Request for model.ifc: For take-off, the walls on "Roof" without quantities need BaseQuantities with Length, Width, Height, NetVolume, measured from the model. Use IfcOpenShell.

First a look at what the model holds.

```python
import ifcopenshell
import ifcopenshell.util.element
import ifcopenshell.util.unit

model = ifcopenshell.open("model.ifc")
print(model.schema)
for unit_type in ("LENGTHUNIT", "AREAUNIT", "VOLUMEUNIT"):
    print(unit_type, ifcopenshell.util.unit.calculate_unit_scale(model, unit_type))
storey = next(s for s in model.by_type("IfcBuildingStorey") if s.Name == "Roof")
walls = [e for e in ifcopenshell.util.element.get_decomposition(storey) if e.is_a("IfcWall")]
for e in sorted(walls, key=lambda e: e.id()):
    print(e.id(), e.is_a(), e.Name, list(ifcopenshell.util.element.get_psets(e, qtos_only=True)), sep=" | ")
```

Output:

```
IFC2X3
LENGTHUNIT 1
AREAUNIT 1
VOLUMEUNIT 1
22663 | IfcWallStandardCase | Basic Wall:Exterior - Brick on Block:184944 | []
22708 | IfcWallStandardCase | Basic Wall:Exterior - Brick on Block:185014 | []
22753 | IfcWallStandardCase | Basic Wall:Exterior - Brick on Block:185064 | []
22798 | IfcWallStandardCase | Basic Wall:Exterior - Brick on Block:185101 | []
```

```python
import ifcopenshell
import ifcopenshell.api.pset
import ifcopenshell.geom
import ifcopenshell.util.element
import ifcopenshell.util.shape
import ifcopenshell.util.unit

model = ifcopenshell.open("model.ifc")
unit_scale = ifcopenshell.util.unit.calculate_unit_scale(model)
volume_scale = ifcopenshell.util.unit.calculate_unit_scale(model, "VOLUMEUNIT")
settings = ifcopenshell.geom.settings()

storey = next(s for s in model.by_type("IfcBuildingStorey") if s.Name == "Roof")
walls = [e for e in ifcopenshell.util.element.get_decomposition(storey) if e.is_a("IfcWall")]

for e in sorted(walls, key=lambda e: e.id()):
    if ifcopenshell.util.element.get_psets(e, qtos_only=True, should_inherit=False):
        continue
    # Geometry comes back in metres, in the element's own axes.
    shape = ifcopenshell.geom.create_shape(settings, e)
    values = {
        "Length": ifcopenshell.util.shape.get_x(shape.geometry) / unit_scale,
        "Width": ifcopenshell.util.shape.get_y(shape.geometry) / unit_scale,
        "Height": ifcopenshell.util.shape.get_z(shape.geometry) / unit_scale,
        "NetVolume": ifcopenshell.util.shape.get_volume(shape.geometry) / volume_scale,
    }
    qto = ifcopenshell.api.pset.add_qto(model, product=e, name="BaseQuantities")
    ifcopenshell.api.pset.edit_qto(model, qto=qto, properties=values)
    print(e.id(), {k: round(v, 3) for k, v in values.items()})

model.write("model-out.ifc")
```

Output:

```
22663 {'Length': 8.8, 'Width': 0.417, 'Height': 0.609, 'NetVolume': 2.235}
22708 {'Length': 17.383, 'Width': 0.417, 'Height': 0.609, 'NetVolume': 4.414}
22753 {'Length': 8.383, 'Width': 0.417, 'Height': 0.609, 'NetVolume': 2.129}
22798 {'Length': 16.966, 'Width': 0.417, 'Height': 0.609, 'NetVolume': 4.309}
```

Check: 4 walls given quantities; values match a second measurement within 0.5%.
